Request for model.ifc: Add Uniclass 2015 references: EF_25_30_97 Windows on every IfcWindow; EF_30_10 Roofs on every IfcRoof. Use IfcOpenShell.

First a look at what the model holds.

```python
import ifcopenshell

model = ifcopenshell.open("model.ifc")
print(model.schema)
print("classifications:", [c.Name for c in model.by_type("IfcClassification")])
for ifc_class in ("IfcDoor", "IfcRoof", "IfcStair", "IfcWall", "IfcWindow"):
    print(ifc_class, len(model.by_type(ifc_class)))
```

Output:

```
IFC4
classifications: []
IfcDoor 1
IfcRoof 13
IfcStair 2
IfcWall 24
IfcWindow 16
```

```python
import ifcopenshell
import ifcopenshell.api.classification

model = ifcopenshell.open("model.ifc")

system = ifcopenshell.api.classification.add_classification(model, classification="Uniclass 2015")

codes = {
    "IfcWindow": ("EF_25_30_97", "Windows"),
    "IfcRoof": ("EF_30_10", "Roofs"),
}
for ifc_class, (code, name) in codes.items():
    products = model.by_type(ifc_class)
    ifcopenshell.api.classification.add_reference(
        model, products=products, classification=system, identification=code, name=name
    )
    print(code, len(products))

model.write("model_v2.ifc")
```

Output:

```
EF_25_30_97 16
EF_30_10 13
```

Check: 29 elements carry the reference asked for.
